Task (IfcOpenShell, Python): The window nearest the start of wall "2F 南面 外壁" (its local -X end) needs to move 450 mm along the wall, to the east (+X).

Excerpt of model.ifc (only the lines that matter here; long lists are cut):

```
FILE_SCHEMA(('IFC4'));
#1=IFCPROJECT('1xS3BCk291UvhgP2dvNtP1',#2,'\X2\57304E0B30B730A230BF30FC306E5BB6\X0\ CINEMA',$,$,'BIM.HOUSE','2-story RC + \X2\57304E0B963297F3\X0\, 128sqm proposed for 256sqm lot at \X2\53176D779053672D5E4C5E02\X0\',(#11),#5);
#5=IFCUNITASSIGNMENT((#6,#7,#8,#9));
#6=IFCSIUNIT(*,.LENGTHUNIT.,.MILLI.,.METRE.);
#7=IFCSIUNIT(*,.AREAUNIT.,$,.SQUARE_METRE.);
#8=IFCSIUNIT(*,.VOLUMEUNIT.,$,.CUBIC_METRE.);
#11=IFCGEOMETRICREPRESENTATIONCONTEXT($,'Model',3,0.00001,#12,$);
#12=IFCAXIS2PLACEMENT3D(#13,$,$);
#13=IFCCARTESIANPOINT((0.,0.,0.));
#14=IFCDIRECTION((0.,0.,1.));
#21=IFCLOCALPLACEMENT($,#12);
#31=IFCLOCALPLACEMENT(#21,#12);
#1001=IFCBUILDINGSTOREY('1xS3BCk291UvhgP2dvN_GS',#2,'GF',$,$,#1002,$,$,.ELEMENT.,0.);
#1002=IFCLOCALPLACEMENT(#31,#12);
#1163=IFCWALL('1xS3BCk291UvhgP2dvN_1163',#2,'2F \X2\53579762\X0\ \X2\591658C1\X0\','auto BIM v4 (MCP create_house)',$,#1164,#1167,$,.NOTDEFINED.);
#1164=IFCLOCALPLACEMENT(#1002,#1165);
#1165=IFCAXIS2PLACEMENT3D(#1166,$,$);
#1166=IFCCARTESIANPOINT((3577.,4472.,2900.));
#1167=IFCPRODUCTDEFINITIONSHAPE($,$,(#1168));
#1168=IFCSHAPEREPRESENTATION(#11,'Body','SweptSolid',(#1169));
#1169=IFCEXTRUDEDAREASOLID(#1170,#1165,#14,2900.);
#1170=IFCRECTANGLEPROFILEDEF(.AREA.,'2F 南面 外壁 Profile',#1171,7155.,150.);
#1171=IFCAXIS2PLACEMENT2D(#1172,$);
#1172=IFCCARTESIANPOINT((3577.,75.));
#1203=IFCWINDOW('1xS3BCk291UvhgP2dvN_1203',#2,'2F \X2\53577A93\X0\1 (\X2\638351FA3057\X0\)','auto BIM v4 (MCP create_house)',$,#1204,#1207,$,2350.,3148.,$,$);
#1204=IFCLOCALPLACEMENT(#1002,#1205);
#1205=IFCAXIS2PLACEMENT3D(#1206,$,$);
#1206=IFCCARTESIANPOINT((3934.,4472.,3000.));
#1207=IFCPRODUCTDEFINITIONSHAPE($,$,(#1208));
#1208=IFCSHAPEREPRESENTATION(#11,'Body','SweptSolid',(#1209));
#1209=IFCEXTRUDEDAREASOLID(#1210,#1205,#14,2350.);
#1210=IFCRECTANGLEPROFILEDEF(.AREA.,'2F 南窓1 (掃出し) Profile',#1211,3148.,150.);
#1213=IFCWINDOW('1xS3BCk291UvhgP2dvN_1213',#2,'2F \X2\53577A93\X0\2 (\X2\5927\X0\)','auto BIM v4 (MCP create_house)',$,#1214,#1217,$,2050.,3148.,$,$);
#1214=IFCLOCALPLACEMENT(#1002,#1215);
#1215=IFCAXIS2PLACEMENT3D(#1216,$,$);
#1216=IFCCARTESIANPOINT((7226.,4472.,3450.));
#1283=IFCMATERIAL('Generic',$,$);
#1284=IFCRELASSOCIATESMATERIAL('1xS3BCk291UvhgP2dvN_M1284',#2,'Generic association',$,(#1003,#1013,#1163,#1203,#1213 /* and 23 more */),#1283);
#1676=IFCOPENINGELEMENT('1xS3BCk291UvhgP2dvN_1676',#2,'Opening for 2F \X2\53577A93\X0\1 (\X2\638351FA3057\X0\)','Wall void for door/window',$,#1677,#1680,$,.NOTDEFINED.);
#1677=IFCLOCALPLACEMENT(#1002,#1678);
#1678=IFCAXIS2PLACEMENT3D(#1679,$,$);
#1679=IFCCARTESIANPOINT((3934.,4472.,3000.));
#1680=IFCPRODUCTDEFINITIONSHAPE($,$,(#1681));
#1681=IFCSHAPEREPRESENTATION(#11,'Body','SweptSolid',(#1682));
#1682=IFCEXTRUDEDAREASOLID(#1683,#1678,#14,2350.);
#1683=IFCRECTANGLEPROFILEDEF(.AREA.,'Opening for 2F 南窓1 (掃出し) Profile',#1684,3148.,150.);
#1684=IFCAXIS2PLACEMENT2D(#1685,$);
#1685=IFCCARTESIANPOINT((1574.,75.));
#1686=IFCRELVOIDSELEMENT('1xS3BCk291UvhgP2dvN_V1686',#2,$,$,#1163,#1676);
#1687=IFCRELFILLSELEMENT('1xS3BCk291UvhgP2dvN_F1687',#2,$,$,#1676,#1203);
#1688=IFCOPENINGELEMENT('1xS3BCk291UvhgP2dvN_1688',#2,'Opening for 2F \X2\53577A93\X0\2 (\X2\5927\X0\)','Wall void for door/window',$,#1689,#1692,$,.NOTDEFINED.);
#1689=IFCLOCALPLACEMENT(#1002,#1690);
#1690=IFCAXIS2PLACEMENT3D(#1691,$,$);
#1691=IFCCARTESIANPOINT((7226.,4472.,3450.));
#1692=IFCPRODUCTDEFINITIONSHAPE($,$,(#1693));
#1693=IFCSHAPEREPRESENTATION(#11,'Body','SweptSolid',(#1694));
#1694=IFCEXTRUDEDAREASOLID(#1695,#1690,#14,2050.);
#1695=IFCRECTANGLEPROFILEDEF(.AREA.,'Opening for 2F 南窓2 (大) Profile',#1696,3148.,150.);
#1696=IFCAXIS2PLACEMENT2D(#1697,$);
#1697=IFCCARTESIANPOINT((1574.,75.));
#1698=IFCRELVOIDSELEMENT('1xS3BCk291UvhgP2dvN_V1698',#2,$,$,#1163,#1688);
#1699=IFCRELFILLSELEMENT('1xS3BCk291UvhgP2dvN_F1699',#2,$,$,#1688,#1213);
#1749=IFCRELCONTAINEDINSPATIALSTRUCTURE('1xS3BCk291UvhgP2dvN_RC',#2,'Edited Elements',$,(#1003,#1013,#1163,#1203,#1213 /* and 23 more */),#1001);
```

```python
import ifcopenshell
import ifcopenshell.api.geometry
import ifcopenshell.util.placement

model = ifcopenshell.open("model.ifc")

window = model.by_guid("1xS3BCk291UvhgP2dvN_1203")
opening = window.FillsVoids[0].RelatingOpeningElement
wall = opening.VoidsElements[0].RelatingBuildingElement

wall_matrix = ifcopenshell.util.placement.get_local_placement(wall.ObjectPlacement)
shift = wall_matrix[:3, 0] * 450.0
before = ifcopenshell.util.placement.get_local_placement(window.ObjectPlacement)[:3, 3].copy()

# The window is not placed relative to its opening, so move both.
for product in (opening, window):
    matrix = ifcopenshell.util.placement.get_local_placement(product.ObjectPlacement)
    matrix[:3, 3] += shift
    ifcopenshell.api.geometry.edit_object_placement(model, product=product, matrix=matrix, is_si=False)

after = ifcopenshell.util.placement.get_local_placement(window.ObjectPlacement)[:3, 3]
print("window moved by", (after - before).round(3) + 0.0)

model.write("model_v2.ifc")
```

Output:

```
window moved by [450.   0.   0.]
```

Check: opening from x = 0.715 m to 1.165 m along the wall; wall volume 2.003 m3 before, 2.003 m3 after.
